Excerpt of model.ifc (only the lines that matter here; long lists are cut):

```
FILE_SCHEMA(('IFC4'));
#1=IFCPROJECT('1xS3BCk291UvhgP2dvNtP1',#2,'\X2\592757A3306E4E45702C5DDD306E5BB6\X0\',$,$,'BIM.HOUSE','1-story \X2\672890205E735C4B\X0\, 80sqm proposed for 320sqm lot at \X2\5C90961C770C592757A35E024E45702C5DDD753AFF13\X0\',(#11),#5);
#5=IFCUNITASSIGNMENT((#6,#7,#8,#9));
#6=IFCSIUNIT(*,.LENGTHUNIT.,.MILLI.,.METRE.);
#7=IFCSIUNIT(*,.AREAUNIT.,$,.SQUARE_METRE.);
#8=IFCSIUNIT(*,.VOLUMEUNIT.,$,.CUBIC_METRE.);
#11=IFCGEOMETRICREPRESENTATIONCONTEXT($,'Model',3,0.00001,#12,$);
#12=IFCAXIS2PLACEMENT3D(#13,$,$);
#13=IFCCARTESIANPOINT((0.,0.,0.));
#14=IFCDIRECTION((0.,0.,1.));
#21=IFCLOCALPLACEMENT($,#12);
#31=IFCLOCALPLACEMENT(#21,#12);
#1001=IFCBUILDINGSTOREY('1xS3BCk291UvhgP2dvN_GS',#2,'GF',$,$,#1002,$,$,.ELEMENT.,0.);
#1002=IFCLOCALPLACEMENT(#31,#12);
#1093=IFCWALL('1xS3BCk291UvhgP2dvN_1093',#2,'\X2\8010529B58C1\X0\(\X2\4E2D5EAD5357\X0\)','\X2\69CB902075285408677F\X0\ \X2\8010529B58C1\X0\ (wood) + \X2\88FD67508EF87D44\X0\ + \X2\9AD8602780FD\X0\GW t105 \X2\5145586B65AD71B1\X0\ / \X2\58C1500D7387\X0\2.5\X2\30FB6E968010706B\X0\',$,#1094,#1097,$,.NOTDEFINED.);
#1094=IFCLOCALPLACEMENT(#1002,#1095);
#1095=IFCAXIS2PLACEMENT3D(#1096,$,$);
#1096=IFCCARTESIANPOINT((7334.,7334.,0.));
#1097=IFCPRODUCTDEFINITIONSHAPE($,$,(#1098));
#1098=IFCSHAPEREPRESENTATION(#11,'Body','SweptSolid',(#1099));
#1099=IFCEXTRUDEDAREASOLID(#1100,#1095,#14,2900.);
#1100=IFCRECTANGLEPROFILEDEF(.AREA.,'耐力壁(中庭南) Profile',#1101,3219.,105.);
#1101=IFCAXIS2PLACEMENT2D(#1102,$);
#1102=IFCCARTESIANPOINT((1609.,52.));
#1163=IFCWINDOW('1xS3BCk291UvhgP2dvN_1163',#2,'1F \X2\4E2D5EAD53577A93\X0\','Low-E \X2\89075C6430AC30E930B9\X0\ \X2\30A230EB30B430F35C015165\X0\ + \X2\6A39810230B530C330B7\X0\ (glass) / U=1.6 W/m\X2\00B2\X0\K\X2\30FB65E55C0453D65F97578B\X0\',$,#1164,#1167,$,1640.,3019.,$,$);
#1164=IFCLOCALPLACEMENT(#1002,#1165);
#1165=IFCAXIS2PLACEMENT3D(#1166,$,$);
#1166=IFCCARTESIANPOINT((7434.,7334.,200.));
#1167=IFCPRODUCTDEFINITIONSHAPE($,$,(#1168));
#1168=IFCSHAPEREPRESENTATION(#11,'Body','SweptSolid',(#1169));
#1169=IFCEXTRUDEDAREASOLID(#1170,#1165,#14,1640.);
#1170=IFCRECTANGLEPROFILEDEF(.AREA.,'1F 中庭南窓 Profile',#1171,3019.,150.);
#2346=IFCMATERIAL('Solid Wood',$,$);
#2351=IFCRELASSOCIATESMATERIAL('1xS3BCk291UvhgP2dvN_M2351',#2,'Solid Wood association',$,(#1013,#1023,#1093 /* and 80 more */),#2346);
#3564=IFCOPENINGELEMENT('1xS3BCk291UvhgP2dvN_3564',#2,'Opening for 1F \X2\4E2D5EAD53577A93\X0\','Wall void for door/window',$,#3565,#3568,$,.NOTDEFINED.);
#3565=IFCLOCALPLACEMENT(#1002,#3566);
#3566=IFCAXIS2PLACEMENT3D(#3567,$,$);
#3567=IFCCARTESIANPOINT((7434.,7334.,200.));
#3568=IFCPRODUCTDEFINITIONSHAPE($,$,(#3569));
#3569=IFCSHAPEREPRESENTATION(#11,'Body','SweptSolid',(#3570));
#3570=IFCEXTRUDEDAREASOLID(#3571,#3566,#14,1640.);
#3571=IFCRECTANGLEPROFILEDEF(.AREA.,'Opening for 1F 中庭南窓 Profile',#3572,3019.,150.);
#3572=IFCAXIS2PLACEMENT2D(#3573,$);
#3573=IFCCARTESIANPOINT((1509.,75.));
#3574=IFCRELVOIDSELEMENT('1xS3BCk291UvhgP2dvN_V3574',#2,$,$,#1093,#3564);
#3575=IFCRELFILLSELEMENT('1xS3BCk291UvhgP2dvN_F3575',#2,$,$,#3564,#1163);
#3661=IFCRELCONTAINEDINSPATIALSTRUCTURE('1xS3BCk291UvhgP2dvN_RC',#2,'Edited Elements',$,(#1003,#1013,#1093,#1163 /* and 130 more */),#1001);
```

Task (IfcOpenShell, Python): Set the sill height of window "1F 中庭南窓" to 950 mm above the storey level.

```python
import numpy as np
import ifcopenshell
import ifcopenshell.api.geometry
import ifcopenshell.geom
import ifcopenshell.util.element
import ifcopenshell.util.placement
import ifcopenshell.util.shape
import ifcopenshell.util.unit

model = ifcopenshell.open("model.ifc")
unit_scale = ifcopenshell.util.unit.calculate_unit_scale(model)

window = model.by_guid("1xS3BCk291UvhgP2dvN_1163")
opening = window.FillsVoids[0].RelatingOpeningElement
storey = ifcopenshell.util.element.get_container(window, ifc_class="IfcBuildingStorey")
level = ifcopenshell.util.placement.get_local_placement(storey.ObjectPlacement)[2, 3]

# The opening's origin need not be at the sill, so measure its lowest point.
shape = ifcopenshell.geom.create_shape(ifcopenshell.geom.settings(), opening)
bottom = ifcopenshell.util.shape.get_shape_bottom_elevation(shape, shape.geometry) / unit_scale
dz = level + 950.0 - bottom

shift = np.array([0.0, 0.0, dz])
# The window is not placed relative to its opening, so move both.
for product in (opening, window):
    matrix = ifcopenshell.util.placement.get_local_placement(product.ObjectPlacement)
    matrix[:3, 3] += shift
    ifcopenshell.api.geometry.edit_object_placement(model, product=product, matrix=matrix, is_si=False)

print(f"moved by {dz * unit_scale:+.3f} m")

model.write("model_v2.ifc")
```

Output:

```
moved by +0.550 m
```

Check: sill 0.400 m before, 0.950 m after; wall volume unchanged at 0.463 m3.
